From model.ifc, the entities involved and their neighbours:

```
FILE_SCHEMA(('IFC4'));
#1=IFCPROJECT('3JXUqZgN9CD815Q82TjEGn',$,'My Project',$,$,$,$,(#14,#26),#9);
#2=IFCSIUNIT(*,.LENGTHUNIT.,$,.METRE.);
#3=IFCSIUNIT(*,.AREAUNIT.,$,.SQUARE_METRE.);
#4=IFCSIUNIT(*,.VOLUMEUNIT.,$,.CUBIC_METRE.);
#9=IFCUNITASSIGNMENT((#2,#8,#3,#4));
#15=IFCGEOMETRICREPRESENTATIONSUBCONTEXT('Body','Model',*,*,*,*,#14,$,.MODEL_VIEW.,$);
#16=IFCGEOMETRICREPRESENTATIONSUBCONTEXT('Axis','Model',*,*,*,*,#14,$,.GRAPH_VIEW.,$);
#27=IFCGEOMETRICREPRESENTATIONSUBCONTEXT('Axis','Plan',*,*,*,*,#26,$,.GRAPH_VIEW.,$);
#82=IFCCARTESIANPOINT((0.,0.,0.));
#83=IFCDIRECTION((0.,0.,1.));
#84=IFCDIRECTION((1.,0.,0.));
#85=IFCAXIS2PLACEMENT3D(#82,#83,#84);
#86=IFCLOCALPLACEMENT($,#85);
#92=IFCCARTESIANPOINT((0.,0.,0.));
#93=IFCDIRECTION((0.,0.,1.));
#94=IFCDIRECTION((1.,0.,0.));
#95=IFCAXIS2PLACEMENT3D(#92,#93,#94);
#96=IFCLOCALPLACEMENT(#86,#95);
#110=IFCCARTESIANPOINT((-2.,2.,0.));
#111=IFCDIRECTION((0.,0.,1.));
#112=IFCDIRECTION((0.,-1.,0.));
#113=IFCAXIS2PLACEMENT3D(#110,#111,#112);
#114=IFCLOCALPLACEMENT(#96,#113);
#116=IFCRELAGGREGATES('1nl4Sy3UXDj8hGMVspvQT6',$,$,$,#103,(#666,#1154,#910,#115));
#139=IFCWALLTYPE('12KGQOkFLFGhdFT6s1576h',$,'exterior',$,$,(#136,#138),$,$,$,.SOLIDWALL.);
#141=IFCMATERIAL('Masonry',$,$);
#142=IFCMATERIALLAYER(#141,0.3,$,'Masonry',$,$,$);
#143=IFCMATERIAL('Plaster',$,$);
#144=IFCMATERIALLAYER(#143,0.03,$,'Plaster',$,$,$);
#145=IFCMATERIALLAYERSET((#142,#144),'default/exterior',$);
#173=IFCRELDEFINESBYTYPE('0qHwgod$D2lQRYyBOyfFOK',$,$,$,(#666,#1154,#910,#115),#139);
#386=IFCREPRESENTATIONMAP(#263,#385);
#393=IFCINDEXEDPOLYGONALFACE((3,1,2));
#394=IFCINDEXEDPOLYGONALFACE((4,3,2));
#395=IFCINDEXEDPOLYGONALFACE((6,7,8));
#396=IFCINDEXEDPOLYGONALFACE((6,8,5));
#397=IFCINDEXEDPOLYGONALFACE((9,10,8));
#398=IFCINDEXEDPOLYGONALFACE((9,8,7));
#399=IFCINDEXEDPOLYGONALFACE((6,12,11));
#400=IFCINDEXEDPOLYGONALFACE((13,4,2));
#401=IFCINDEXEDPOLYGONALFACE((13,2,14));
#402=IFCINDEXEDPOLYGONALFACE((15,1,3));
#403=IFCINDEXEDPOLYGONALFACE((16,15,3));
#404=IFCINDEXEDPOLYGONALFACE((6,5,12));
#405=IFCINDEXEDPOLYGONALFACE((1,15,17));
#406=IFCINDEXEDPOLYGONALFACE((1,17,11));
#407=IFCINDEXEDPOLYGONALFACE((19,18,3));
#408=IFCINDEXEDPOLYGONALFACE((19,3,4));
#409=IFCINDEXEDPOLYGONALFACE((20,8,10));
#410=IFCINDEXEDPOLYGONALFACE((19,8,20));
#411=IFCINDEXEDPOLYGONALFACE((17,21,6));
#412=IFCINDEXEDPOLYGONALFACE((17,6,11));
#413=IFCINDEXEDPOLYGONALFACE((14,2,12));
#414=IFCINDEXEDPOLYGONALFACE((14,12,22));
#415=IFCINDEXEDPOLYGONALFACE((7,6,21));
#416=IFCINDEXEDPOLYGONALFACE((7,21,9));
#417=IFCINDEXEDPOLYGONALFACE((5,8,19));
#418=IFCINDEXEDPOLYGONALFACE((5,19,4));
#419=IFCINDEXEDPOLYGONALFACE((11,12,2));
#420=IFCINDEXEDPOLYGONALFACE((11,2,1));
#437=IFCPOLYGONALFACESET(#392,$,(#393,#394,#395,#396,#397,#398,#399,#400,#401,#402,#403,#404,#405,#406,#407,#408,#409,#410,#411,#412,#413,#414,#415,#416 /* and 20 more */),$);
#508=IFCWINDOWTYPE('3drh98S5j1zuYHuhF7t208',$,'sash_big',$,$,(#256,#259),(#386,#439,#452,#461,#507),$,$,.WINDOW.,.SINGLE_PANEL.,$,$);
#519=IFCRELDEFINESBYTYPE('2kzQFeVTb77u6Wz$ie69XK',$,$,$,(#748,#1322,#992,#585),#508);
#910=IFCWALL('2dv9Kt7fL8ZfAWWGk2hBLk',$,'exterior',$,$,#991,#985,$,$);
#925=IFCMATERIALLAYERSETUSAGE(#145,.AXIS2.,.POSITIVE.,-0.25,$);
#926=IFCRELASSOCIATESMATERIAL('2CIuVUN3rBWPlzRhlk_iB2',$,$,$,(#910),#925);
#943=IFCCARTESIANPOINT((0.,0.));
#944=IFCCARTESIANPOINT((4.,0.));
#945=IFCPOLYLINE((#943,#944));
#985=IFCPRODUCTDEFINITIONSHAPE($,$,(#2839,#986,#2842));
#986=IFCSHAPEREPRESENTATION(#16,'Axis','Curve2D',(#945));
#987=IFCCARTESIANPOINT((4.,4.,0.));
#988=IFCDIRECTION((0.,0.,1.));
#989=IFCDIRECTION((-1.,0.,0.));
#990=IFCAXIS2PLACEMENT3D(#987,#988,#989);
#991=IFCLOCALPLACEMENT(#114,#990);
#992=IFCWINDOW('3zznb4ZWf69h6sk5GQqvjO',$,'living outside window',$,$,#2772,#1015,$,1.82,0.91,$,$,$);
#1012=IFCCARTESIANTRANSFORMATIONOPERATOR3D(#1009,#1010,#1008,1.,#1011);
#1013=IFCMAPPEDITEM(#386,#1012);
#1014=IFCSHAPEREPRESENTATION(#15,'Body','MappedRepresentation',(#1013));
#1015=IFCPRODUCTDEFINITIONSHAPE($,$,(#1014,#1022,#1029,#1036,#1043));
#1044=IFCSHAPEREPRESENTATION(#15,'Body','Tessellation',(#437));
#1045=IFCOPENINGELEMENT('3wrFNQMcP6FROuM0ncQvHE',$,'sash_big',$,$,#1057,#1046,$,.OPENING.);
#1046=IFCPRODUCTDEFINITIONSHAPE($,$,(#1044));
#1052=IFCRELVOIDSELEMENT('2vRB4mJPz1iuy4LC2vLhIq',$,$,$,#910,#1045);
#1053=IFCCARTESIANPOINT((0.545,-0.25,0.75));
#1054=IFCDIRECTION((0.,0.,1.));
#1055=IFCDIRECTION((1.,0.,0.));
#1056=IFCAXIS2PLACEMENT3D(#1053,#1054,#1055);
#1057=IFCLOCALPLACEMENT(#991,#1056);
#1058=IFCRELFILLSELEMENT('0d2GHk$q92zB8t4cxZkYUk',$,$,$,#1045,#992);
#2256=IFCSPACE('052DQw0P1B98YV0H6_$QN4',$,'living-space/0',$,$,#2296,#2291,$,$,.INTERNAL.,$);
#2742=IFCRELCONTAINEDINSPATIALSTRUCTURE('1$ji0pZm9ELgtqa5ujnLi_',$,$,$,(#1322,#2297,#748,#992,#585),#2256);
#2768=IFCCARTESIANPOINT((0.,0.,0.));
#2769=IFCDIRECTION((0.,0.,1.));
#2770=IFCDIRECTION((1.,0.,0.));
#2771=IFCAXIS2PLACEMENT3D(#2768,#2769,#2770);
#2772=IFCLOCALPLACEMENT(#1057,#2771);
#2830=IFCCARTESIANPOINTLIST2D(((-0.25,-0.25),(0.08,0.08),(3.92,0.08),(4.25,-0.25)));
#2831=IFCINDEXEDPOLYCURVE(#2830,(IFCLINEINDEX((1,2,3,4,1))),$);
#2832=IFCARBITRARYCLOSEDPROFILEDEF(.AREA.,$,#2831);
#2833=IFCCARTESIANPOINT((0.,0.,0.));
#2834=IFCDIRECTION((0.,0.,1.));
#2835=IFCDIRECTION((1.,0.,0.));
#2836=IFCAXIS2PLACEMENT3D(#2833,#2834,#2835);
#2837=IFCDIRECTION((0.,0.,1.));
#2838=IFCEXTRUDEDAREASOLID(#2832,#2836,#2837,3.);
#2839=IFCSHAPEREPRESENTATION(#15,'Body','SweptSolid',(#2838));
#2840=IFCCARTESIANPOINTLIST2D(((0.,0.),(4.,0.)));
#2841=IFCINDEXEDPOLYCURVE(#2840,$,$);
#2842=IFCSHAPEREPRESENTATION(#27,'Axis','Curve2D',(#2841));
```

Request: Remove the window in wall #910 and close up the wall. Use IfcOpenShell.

```python
import ifcopenshell
import ifcopenshell.api.feature
import ifcopenshell.api.root
import ifcopenshell.geom
import ifcopenshell.util.shape

model = ifcopenshell.open("model.ifc")
settings = ifcopenshell.geom.settings()


def volume(element):
    """Net volume in cubic metres, openings subtracted."""
    shape = ifcopenshell.geom.create_shape(settings, element)
    return ifcopenshell.util.shape.get_volume(shape.geometry)


window = model.by_guid("3zznb4ZWf69h6sk5GQqvjO")
opening = window.FillsVoids[0].RelatingOpeningElement
wall = opening.VoidsElements[0].RelatingBuildingElement
before = volume(wall)

ifcopenshell.api.root.remove_product(model, product=window)
ifcopenshell.api.feature.remove_feature(model, feature=opening)

after = volume(wall)

print(f"wall volume {before:.3f} -> {after:.3f} m3")

model.write("model-out.ifc")
```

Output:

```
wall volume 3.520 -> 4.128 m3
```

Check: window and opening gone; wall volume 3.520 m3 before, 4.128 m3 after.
